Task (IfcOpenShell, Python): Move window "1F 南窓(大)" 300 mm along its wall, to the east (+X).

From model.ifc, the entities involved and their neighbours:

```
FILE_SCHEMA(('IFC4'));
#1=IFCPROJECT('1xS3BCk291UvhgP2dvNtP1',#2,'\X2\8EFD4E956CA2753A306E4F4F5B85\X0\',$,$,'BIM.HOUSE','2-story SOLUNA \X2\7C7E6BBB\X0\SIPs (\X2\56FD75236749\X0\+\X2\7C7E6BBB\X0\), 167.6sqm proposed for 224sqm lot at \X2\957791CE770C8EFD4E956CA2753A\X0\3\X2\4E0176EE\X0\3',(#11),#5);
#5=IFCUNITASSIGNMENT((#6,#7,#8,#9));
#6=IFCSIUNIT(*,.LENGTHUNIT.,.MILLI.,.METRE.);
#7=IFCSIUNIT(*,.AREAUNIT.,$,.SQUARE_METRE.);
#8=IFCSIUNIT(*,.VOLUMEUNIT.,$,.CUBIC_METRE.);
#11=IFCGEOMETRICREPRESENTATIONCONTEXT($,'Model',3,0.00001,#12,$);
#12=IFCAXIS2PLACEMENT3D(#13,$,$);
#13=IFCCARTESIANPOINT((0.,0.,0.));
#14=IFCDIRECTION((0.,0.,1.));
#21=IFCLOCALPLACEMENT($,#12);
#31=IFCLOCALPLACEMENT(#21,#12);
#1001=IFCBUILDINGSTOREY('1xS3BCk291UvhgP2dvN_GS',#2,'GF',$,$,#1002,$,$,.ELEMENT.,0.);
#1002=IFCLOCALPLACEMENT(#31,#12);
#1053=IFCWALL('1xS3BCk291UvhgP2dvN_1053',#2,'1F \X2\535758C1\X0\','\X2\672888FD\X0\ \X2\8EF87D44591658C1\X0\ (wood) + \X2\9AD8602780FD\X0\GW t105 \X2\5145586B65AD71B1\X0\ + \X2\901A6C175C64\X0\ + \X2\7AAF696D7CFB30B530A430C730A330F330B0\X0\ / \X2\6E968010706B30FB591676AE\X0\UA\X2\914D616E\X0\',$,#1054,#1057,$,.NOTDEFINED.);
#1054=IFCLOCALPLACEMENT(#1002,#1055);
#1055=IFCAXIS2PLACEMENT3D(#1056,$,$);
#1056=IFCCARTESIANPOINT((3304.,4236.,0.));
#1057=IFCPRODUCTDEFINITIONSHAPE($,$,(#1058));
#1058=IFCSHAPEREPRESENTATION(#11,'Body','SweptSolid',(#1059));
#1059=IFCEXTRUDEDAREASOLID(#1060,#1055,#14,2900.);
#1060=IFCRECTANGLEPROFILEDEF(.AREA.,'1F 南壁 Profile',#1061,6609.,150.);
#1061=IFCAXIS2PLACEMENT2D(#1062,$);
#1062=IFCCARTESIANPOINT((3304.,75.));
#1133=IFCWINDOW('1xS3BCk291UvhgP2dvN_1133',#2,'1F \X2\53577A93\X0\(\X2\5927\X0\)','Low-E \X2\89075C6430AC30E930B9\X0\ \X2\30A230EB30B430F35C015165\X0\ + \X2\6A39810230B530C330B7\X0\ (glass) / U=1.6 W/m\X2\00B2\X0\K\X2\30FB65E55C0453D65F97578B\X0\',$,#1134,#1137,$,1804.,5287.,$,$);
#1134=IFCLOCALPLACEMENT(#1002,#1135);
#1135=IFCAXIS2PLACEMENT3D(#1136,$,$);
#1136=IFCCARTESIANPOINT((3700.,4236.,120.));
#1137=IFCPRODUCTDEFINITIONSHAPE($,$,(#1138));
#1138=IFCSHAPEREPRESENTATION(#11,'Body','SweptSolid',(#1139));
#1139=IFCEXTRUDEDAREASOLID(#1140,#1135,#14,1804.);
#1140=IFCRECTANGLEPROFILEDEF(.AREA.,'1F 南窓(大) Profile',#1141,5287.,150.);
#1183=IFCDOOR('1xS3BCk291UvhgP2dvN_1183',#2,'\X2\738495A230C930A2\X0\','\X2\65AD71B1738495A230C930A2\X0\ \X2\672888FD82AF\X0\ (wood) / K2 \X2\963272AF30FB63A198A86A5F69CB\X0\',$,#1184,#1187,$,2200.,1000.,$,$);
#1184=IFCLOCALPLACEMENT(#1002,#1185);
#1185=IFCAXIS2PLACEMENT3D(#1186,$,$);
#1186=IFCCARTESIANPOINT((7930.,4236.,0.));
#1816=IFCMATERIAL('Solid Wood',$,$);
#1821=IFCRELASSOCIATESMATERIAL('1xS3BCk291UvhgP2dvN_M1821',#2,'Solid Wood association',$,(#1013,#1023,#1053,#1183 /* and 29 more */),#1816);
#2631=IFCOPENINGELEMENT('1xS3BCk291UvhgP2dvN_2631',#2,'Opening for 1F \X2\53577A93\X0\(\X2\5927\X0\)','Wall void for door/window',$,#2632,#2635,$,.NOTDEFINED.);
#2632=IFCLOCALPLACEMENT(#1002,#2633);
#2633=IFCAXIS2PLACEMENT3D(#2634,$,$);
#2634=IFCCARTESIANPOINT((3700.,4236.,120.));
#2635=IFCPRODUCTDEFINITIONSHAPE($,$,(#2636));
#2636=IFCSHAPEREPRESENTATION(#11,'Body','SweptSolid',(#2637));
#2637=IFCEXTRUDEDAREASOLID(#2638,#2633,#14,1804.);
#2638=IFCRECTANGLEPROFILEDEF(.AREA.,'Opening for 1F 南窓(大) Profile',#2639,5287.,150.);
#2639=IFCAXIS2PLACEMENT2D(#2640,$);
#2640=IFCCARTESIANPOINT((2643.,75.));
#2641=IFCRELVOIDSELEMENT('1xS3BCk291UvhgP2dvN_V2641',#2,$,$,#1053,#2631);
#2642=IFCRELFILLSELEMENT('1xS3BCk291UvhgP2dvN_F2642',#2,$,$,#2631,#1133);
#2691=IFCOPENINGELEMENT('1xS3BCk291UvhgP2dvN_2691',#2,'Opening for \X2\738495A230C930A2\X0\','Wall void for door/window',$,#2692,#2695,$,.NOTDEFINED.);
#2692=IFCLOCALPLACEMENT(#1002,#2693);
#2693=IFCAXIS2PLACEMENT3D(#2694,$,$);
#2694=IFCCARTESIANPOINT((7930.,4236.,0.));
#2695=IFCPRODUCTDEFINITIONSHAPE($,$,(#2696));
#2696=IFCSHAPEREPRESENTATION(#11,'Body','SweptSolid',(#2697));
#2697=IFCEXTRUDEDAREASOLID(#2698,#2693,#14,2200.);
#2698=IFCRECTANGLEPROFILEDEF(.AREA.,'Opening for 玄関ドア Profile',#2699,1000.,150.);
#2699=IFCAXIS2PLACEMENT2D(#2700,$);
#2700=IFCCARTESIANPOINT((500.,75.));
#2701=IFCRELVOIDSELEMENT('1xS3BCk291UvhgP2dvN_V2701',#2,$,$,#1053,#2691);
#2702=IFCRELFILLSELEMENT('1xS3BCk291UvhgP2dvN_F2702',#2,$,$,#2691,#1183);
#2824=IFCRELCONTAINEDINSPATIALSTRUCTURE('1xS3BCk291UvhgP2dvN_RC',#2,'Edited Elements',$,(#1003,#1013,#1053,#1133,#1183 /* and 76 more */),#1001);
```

```python
import ifcopenshell
import ifcopenshell.api.geometry
import ifcopenshell.util.placement

model = ifcopenshell.open("model.ifc")

window = model.by_guid("1xS3BCk291UvhgP2dvN_1133")
opening = window.FillsVoids[0].RelatingOpeningElement
wall = opening.VoidsElements[0].RelatingBuildingElement

wall_matrix = ifcopenshell.util.placement.get_local_placement(wall.ObjectPlacement)
shift = wall_matrix[:3, 0] * 300.0
before = ifcopenshell.util.placement.get_local_placement(window.ObjectPlacement)[:3, 3].copy()

# The window is not placed relative to its opening, so move both.
for product in (opening, window):
    matrix = ifcopenshell.util.placement.get_local_placement(product.ObjectPlacement)
    matrix[:3, 3] += shift
    ifcopenshell.api.geometry.edit_object_placement(model, product=product, matrix=matrix, is_si=False)

after = ifcopenshell.util.placement.get_local_placement(window.ObjectPlacement)[:3, 3]
print("window moved by", (after - before).round(3) + 0.0)

model.write("model_rev.ifc")
```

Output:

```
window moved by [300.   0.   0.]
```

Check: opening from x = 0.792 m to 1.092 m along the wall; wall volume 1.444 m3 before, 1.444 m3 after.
